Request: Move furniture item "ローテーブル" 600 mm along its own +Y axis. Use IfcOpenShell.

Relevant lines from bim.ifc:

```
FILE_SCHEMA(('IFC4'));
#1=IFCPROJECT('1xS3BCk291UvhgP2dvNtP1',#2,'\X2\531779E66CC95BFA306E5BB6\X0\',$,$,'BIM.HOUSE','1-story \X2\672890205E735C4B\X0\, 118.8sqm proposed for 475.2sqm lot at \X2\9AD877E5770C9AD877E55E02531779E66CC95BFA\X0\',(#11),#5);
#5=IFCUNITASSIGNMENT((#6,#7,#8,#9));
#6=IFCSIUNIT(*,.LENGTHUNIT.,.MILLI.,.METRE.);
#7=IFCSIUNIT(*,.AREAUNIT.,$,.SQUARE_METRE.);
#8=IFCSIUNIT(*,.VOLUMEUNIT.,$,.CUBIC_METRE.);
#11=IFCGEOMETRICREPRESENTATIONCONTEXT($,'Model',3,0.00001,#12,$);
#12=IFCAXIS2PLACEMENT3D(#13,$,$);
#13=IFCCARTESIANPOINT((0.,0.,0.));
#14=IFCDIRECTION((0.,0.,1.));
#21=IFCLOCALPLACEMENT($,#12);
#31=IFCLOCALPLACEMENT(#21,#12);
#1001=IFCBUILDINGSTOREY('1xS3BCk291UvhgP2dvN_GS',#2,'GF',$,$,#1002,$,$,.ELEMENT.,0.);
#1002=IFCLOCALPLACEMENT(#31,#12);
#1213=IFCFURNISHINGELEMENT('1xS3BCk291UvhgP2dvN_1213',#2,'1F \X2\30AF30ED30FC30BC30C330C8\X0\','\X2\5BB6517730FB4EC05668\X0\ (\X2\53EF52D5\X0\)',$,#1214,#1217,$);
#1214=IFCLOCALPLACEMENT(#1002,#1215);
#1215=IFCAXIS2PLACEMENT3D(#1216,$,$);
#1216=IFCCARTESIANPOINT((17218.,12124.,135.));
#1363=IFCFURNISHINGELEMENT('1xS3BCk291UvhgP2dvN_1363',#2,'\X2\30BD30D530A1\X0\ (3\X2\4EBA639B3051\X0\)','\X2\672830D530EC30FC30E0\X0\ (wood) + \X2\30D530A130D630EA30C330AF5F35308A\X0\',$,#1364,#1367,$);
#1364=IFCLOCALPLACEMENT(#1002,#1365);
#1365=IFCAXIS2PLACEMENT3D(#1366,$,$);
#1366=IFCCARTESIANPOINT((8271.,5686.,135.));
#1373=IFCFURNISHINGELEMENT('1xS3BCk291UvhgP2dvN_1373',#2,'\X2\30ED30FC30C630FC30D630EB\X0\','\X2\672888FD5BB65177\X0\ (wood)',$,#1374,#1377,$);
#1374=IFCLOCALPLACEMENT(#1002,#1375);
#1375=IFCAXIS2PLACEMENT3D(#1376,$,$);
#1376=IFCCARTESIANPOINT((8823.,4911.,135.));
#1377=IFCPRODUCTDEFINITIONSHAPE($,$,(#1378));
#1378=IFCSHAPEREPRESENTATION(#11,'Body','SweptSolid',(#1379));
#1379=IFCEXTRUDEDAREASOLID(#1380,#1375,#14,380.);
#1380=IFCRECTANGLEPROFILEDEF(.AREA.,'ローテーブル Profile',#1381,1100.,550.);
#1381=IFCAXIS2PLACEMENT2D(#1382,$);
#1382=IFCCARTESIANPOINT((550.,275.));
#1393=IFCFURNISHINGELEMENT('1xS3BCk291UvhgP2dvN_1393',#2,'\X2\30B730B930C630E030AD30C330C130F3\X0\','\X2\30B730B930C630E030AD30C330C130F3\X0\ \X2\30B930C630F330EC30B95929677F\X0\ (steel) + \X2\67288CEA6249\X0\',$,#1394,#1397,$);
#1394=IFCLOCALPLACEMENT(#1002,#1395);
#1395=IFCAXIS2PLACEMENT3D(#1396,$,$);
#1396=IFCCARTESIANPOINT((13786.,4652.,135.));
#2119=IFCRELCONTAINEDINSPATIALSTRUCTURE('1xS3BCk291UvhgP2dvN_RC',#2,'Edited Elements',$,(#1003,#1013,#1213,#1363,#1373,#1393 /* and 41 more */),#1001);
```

```python
import ifcopenshell
import ifcopenshell.api.geometry
import ifcopenshell.util.placement
import ifcopenshell.util.unit

model = ifcopenshell.open("bim.ifc")
unit_scale = ifcopenshell.util.unit.calculate_unit_scale(model)

item = model.by_guid("1xS3BCk291UvhgP2dvN_1373")
matrix = ifcopenshell.util.placement.get_local_placement(item.ObjectPlacement)
matrix[:3, 3] += matrix[:3, 1] * 0.6 / unit_scale
ifcopenshell.api.geometry.edit_object_placement(model, product=item, matrix=matrix, is_si=False)

print(ifcopenshell.util.placement.get_local_placement(item.ObjectPlacement).round(3) + 0.0)

model.write("bim_v2.ifc")
```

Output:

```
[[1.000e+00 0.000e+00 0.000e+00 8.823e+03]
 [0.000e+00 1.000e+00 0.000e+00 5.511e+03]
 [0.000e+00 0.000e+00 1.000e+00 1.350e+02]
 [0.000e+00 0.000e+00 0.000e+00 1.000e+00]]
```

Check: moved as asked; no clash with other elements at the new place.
